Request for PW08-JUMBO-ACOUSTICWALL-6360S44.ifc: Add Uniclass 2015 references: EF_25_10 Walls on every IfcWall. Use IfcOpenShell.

First a look at what the model holds.

```python
import ifcopenshell

model = ifcopenshell.open("PW08-JUMBO-ACOUSTICWALL-6360S44.ifc")
print(model.schema)
print("classifications:", [c.Name for c in model.by_type("IfcClassification")])
for ifc_class in ("IfcDoor", "IfcRoof", "IfcStair", "IfcWall", "IfcWindow"):
    print(ifc_class, len(model.by_type(ifc_class)))
```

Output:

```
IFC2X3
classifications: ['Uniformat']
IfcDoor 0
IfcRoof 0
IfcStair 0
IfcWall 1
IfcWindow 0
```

```python
import ifcopenshell
import ifcopenshell.api.classification

model = ifcopenshell.open("PW08-JUMBO-ACOUSTICWALL-6360S44.ifc")

# IFC2X3 requires Source and Edition and has no link from the project to the system.
system = model.create_entity("IfcClassification", Source="NBS", Edition="2015", Name="Uniclass 2015")

codes = {
    "IfcWall": ("EF_25_10", "Walls"),
}
for ifc_class, (code, name) in codes.items():
    products = model.by_type(ifc_class)
    ifcopenshell.api.classification.add_reference(
        model, products=products, classification=system, identification=code, name=name
    )
    print(code, len(products))

model.write("PW08-JUMBO-ACOUSTICWALL-6360S44_rev.ifc")
```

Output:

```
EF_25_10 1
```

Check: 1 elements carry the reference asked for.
